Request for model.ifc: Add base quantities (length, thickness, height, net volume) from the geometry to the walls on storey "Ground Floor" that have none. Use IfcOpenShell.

First a look at what the model holds.

```python
import ifcopenshell
import ifcopenshell.util.element
import ifcopenshell.util.unit

model = ifcopenshell.open("model.ifc")
print(model.schema)
for unit_type in ("LENGTHUNIT", "AREAUNIT", "VOLUMEUNIT"):
    print(unit_type, ifcopenshell.util.unit.calculate_unit_scale(model, unit_type))
storey = next(s for s in model.by_type("IfcBuildingStorey") if s.Name == "Ground Floor")
walls = [e for e in ifcopenshell.util.element.get_decomposition(storey) if e.is_a("IfcWall")]
for e in sorted(walls, key=lambda e: e.id()):
    print(e.id(), e.is_a(), e.Name, list(ifcopenshell.util.element.get_psets(e, qtos_only=True)), sep=" | ")
```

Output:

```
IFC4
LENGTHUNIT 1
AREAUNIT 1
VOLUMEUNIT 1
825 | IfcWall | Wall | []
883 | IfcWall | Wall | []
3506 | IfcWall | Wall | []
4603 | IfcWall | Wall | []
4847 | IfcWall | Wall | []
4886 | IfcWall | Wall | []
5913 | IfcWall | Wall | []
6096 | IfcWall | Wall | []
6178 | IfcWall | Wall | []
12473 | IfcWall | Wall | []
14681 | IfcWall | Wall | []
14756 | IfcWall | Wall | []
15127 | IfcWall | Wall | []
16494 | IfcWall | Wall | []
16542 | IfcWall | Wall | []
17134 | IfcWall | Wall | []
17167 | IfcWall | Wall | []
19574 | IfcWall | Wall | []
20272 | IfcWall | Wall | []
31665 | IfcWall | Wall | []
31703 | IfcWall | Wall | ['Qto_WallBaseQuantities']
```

```python
import ifcopenshell
import ifcopenshell.api.pset
import ifcopenshell.geom
import ifcopenshell.util.element
import ifcopenshell.util.shape
import ifcopenshell.util.unit

model = ifcopenshell.open("model.ifc")
unit_scale = ifcopenshell.util.unit.calculate_unit_scale(model)
volume_scale = ifcopenshell.util.unit.calculate_unit_scale(model, "VOLUMEUNIT")
settings = ifcopenshell.geom.settings()

storey = next(s for s in model.by_type("IfcBuildingStorey") if s.Name == "Ground Floor")
walls = [e for e in ifcopenshell.util.element.get_decomposition(storey) if e.is_a("IfcWall")]

for e in sorted(walls, key=lambda e: e.id()):
    if ifcopenshell.util.element.get_psets(e, qtos_only=True, should_inherit=False):
        continue
    # Geometry comes back in metres, in the element's own axes.
    shape = ifcopenshell.geom.create_shape(settings, e)
    values = {
        "Length": ifcopenshell.util.shape.get_x(shape.geometry) / unit_scale,
        "Width": ifcopenshell.util.shape.get_y(shape.geometry) / unit_scale,
        "Height": ifcopenshell.util.shape.get_z(shape.geometry) / unit_scale,
        "NetVolume": ifcopenshell.util.shape.get_volume(shape.geometry) / volume_scale,
    }
    qto = ifcopenshell.api.pset.add_qto(model, product=e, name="Qto_WallBaseQuantities")
    ifcopenshell.api.pset.edit_qto(model, qto=qto, properties=values)
    print(e.id(), {k: round(v, 3) for k, v in values.items()})

model.write("model_updated.ifc")
```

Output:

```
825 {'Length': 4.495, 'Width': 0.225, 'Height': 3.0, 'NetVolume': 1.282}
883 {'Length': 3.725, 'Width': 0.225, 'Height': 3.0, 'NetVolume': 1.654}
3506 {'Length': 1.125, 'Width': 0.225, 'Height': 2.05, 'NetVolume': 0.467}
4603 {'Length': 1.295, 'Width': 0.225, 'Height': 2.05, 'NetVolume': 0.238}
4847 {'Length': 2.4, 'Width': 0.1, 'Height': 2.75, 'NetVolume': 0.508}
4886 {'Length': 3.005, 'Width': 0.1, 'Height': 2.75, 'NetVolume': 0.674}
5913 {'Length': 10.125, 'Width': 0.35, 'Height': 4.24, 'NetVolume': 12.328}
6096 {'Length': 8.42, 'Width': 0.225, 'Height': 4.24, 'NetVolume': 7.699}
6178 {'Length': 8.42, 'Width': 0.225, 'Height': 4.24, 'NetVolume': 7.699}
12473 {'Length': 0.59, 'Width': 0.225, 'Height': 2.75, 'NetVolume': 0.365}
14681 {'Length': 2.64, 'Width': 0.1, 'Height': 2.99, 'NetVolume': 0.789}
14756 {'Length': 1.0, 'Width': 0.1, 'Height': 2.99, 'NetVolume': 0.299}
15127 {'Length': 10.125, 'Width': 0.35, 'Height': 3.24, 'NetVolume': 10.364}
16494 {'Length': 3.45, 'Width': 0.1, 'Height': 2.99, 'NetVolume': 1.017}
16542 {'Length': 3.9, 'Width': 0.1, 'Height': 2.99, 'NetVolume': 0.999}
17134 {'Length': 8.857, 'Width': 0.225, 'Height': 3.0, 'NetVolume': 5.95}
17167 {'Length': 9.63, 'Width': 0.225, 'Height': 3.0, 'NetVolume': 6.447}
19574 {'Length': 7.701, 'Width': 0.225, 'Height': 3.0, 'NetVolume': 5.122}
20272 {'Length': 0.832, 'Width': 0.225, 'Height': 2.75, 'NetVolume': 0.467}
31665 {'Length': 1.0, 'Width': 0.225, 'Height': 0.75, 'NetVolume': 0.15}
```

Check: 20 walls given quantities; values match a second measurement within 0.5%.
